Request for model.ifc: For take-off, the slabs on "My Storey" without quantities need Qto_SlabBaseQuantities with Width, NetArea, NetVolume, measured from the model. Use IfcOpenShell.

First a look at what the model holds.

```python
import ifcopenshell
import ifcopenshell.util.element
import ifcopenshell.util.unit

model = ifcopenshell.open("model.ifc")
print(model.schema)
for unit_type in ("LENGTHUNIT", "AREAUNIT", "VOLUMEUNIT"):
    print(unit_type, ifcopenshell.util.unit.calculate_unit_scale(model, unit_type))
storey = next(s for s in model.by_type("IfcBuildingStorey") if s.Name == "My Storey")
slabs = [e for e in ifcopenshell.util.element.get_decomposition(storey) if e.is_a("IfcSlab")]
for e in sorted(slabs, key=lambda e: e.id()):
    print(e.id(), e.is_a(), e.Name, list(ifcopenshell.util.element.get_psets(e, qtos_only=True)), sep=" | ")
```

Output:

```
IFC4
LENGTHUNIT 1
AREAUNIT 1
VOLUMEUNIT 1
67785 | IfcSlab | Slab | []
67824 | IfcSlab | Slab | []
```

```python
import ifcopenshell
import ifcopenshell.api.pset
import ifcopenshell.geom
import ifcopenshell.util.element
import ifcopenshell.util.shape
import ifcopenshell.util.unit

model = ifcopenshell.open("model.ifc")
unit_scale = ifcopenshell.util.unit.calculate_unit_scale(model)
area_scale = ifcopenshell.util.unit.calculate_unit_scale(model, "AREAUNIT")
volume_scale = ifcopenshell.util.unit.calculate_unit_scale(model, "VOLUMEUNIT")
settings = ifcopenshell.geom.settings()

storey = next(s for s in model.by_type("IfcBuildingStorey") if s.Name == "My Storey")
slabs = [e for e in ifcopenshell.util.element.get_decomposition(storey) if e.is_a("IfcSlab")]

for e in sorted(slabs, key=lambda e: e.id()):
    if ifcopenshell.util.element.get_psets(e, qtos_only=True, should_inherit=False):
        continue
    # Geometry comes back in metres, in the element's own axes.
    shape = ifcopenshell.geom.create_shape(settings, e)
    values = {
        "Width": ifcopenshell.util.shape.get_z(shape.geometry) / unit_scale,
        "NetArea": ifcopenshell.util.shape.get_footprint_area(shape.geometry) / area_scale,
        "NetVolume": ifcopenshell.util.shape.get_volume(shape.geometry) / volume_scale,
    }
    qto = ifcopenshell.api.pset.add_qto(model, product=e, name="Qto_SlabBaseQuantities")
    ifcopenshell.api.pset.edit_qto(model, qto=qto, properties=values)
    print(e.id(), {k: round(v, 3) for k, v in values.items()})

model.write("model_updated.ifc")
```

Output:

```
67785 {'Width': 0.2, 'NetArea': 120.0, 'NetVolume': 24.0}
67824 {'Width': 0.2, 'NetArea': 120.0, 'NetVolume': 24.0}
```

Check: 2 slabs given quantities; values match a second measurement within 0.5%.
